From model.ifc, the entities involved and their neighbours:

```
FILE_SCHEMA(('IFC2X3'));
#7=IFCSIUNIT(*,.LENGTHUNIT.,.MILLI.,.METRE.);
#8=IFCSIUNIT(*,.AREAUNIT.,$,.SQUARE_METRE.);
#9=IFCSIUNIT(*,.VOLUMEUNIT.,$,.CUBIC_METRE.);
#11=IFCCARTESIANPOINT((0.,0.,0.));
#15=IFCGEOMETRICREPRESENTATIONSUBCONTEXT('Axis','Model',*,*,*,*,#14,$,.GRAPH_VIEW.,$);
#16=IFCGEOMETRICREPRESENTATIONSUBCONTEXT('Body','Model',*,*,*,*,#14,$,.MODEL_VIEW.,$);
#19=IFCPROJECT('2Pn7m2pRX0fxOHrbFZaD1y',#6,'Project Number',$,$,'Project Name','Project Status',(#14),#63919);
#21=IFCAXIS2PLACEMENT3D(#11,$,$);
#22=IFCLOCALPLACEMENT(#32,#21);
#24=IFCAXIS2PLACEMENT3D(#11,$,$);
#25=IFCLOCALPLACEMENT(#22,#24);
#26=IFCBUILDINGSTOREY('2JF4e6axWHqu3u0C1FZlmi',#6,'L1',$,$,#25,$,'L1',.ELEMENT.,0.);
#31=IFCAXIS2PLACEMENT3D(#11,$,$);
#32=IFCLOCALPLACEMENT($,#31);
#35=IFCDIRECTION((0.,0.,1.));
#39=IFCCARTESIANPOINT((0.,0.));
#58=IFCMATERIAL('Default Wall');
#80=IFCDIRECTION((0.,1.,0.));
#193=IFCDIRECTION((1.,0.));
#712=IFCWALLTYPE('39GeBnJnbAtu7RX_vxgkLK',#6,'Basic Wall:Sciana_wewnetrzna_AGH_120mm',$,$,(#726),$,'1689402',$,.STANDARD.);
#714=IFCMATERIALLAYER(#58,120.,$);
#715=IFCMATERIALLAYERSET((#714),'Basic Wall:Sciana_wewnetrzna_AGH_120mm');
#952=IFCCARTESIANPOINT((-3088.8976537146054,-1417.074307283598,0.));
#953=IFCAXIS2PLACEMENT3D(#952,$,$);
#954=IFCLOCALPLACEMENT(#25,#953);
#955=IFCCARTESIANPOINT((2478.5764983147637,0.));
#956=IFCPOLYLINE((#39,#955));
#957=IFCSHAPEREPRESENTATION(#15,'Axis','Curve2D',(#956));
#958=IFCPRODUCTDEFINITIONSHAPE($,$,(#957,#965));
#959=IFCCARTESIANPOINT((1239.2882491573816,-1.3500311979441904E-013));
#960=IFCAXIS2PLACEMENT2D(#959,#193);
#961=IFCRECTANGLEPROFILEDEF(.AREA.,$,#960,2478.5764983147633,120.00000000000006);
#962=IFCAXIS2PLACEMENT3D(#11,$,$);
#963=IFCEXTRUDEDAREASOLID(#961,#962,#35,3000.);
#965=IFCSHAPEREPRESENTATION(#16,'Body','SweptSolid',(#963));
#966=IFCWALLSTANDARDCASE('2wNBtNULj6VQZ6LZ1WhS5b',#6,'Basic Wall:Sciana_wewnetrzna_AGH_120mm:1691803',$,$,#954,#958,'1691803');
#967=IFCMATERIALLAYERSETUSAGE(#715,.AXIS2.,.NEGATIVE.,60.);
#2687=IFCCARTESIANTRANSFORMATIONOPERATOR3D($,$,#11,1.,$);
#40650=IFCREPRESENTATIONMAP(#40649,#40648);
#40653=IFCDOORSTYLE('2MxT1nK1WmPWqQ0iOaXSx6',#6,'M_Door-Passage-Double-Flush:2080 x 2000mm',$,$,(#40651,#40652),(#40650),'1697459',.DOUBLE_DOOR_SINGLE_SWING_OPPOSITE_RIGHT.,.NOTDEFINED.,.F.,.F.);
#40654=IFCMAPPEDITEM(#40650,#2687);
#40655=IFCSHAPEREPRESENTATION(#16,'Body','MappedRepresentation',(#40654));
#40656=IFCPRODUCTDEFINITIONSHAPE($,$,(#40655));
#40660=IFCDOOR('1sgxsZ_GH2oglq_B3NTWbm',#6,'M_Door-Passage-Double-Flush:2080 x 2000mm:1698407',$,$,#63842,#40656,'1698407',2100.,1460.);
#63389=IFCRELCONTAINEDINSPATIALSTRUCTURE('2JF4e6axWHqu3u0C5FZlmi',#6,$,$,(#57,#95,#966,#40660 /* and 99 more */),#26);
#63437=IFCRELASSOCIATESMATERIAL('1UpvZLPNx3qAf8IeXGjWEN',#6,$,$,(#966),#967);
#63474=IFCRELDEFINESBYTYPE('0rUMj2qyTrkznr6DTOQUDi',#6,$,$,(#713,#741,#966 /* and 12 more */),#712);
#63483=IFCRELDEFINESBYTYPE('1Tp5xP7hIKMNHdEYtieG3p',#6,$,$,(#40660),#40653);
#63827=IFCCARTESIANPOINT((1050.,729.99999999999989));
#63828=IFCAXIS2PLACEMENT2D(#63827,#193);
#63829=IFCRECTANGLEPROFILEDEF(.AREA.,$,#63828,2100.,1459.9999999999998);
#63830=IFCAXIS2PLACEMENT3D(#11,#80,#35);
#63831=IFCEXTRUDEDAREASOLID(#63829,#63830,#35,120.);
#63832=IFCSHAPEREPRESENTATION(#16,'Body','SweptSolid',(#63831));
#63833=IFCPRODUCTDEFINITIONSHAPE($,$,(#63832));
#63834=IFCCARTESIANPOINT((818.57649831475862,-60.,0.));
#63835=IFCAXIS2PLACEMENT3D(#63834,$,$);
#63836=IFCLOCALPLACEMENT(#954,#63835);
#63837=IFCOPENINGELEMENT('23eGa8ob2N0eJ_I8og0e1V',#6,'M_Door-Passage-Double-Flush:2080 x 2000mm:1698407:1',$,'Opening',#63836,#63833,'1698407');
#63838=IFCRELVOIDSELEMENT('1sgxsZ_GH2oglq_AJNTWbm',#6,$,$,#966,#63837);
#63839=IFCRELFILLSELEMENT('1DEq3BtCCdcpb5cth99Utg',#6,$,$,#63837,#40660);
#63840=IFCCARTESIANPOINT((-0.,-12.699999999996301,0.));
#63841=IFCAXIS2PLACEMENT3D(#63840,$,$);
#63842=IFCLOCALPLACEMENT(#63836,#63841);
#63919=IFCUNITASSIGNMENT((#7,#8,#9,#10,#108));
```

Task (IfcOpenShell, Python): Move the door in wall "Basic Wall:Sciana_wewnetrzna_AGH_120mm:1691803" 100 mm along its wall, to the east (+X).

```python
import ifcopenshell
import ifcopenshell.api.geometry
import ifcopenshell.util.placement
import ifcopenshell.util.unit

model = ifcopenshell.open("model.ifc")
unit_scale = ifcopenshell.util.unit.calculate_unit_scale(model)

door = model.by_guid("1sgxsZ_GH2oglq_B3NTWbm")
opening = door.FillsVoids[0].RelatingOpeningElement
wall = opening.VoidsElements[0].RelatingBuildingElement

wall_matrix = ifcopenshell.util.placement.get_local_placement(wall.ObjectPlacement)
shift = wall_matrix[:3, 0] * 0.1 / unit_scale
before = ifcopenshell.util.placement.get_local_placement(door.ObjectPlacement)[:3, 3].copy()

# The door is placed relative to its opening, so it follows when the opening moves.
matrix = ifcopenshell.util.placement.get_local_placement(opening.ObjectPlacement)
matrix[:3, 3] += shift
ifcopenshell.api.geometry.edit_object_placement(
    model, product=opening, matrix=matrix, is_si=False, should_transform_children=True
)

after = ifcopenshell.util.placement.get_local_placement(door.ObjectPlacement)[:3, 3]
print("door moved by", (after - before).round(3) + 0.0)

model.write("model_rev.ifc")
```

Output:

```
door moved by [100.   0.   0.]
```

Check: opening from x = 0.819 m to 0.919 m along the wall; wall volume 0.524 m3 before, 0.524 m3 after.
